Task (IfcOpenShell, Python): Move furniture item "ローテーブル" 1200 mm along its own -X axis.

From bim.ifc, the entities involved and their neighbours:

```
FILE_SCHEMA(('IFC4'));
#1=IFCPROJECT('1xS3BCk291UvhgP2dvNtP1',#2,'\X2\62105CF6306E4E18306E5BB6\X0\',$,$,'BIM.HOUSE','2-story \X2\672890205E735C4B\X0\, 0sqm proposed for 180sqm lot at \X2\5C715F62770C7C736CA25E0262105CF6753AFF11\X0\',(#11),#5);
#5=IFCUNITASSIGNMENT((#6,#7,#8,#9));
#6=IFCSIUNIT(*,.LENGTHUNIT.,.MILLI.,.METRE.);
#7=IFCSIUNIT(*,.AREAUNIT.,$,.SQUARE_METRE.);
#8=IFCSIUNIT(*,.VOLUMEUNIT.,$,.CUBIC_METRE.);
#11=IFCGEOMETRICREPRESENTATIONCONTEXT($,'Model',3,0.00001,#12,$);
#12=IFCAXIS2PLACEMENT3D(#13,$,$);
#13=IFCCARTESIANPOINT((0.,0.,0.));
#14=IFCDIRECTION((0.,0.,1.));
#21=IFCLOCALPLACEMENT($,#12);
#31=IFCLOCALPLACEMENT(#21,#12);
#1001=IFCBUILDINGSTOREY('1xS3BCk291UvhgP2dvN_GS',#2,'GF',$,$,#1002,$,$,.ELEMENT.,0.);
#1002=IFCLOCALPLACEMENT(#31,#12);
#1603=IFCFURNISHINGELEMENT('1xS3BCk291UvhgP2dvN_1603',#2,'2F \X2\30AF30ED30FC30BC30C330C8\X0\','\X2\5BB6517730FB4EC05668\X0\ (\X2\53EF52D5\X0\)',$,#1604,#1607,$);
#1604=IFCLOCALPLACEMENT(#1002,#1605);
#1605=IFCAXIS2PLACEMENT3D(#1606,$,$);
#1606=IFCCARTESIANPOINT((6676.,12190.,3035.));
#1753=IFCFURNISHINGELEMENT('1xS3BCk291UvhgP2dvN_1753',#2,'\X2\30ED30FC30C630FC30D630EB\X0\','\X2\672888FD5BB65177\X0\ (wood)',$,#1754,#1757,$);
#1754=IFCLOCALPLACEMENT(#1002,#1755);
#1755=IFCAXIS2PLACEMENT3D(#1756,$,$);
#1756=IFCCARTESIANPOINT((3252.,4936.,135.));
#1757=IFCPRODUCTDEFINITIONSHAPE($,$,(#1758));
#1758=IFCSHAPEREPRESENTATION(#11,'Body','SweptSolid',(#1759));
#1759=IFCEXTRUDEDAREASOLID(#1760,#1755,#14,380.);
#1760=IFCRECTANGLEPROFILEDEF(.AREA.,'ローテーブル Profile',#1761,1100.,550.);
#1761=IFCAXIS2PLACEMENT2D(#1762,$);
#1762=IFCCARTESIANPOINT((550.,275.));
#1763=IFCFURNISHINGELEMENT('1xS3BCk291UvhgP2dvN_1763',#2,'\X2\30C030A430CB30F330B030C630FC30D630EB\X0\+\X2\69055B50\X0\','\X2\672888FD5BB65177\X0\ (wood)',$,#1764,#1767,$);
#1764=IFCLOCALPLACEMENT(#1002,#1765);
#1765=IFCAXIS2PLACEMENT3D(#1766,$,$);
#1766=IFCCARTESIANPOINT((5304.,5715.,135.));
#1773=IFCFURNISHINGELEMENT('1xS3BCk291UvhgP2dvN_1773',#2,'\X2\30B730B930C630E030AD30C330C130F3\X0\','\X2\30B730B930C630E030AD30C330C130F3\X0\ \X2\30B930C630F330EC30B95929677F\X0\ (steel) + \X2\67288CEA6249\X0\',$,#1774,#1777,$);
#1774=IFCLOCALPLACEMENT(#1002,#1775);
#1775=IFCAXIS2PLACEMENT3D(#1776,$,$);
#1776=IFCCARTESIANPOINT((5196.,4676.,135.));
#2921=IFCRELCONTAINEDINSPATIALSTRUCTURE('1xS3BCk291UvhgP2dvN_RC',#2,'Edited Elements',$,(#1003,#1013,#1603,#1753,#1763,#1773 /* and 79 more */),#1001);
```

```python
import ifcopenshell
import ifcopenshell.api.geometry
import ifcopenshell.util.placement

model = ifcopenshell.open("bim.ifc")

item = model.by_id(1753)
matrix = ifcopenshell.util.placement.get_local_placement(item.ObjectPlacement)
matrix[:3, 3] -= matrix[:3, 0] * 1200.0
ifcopenshell.api.geometry.edit_object_placement(model, product=item, matrix=matrix, is_si=False)

print(ifcopenshell.util.placement.get_local_placement(item.ObjectPlacement).round(3) + 0.0)

model.write("bim_updated.ifc")
```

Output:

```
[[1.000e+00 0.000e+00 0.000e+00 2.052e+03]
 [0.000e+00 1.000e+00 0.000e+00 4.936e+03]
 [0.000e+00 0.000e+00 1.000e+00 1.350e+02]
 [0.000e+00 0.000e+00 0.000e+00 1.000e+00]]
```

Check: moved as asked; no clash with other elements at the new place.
